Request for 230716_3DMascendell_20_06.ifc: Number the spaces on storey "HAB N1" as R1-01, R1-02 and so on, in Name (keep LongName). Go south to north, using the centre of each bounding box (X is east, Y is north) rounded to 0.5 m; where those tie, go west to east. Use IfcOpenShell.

First a look at what the model holds.

```python
import ifcopenshell
import ifcopenshell.util.element
import ifcopenshell.util.placement

model = ifcopenshell.open("230716_3DMascendell_20_06.ifc")
print(model.schema)
storey = next(s for s in model.by_type("IfcBuildingStorey") if s.Name == "HAB N1")
spaces = [e for e in ifcopenshell.util.element.get_decomposition(storey) if e.is_a("IfcSpace")]
for e in sorted(spaces, key=lambda e: e.id()):
    origin = ifcopenshell.util.placement.get_local_placement(e.ObjectPlacement)[:3, 3]
    print(e.id(), e.Name, e.LongName, origin.round(2) + 0.0, sep=" | ")
```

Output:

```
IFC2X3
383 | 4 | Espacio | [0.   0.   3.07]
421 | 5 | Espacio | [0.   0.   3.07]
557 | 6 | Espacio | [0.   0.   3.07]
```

```python
import ifcopenshell
import ifcopenshell.geom
import ifcopenshell.util.element
import ifcopenshell.util.shape

model = ifcopenshell.open("230716_3DMascendell_20_06.ifc")
settings = ifcopenshell.geom.settings()
settings.set("use-world-coords", True)


def centre(element):
    shape = ifcopenshell.geom.create_shape(settings, element)
    return ifcopenshell.util.shape.get_bbox_centroid(shape.geometry)


storey = next(s for s in model.by_type("IfcBuildingStorey") if s.Name == "HAB N1")
spaces = [e for e in ifcopenshell.util.element.get_decomposition(storey) if e.is_a("IfcSpace")]

# Insertion points can sit at a corner or the storey origin, so sort by the geometry (in metres).
centres = {e: centre(e) for e in spaces}
spaces.sort(key=lambda e: (round(centres[e][1] / 0.5), centres[e][0]))

for i, e in enumerate(spaces, start=1):
    number = f"R1-{i:02d}"
    e.Name = number
    print(e.id(), number)

model.write("230716_3DMascendell_20_06_rev.ifc")
```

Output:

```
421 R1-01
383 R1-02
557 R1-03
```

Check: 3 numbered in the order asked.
